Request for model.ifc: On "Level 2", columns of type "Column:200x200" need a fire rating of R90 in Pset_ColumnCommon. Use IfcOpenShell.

First a look at what the model holds.

```python
import ifcopenshell
import ifcopenshell.util.element

model = ifcopenshell.open("model.ifc")
print(model.schema)
storey = next(s for s in model.by_type("IfcBuildingStorey") if s.Name == "Level 2")
columns = [e for e in ifcopenshell.util.element.get_decomposition(storey) if e.is_a("IfcColumn")]
seen = {}
for e in columns:
    element_type = ifcopenshell.util.element.get_type(e)
    key = (element_type.Name if element_type != e and element_type else None, ifcopenshell.util.element.get_pset(e, "Pset_ColumnCommon", "FireRating"))
    seen[key] = seen.get(key, 0) + 1
for (name, value), count in sorted(seen.items(), key=str):
    print(count, "x", name, "|", value)
```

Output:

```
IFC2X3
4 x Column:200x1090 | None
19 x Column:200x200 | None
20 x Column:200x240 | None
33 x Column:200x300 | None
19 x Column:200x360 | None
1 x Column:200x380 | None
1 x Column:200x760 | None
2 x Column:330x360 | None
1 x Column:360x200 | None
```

```python
import ifcopenshell
import ifcopenshell.api.pset
import ifcopenshell.util.element

model = ifcopenshell.open("model.ifc")

storey = next(s for s in model.by_type("IfcBuildingStorey") if s.Name == "Level 2")
columns = [e for e in ifcopenshell.util.element.get_decomposition(storey) if e.is_a("IfcColumn")]

count = 0
for e in columns:
    element_type = ifcopenshell.util.element.get_type(e)
    if element_type in (None, e) or element_type.Name != "Column:200x200":
        continue
    # add_pset returns the element's existing set when there is one.
    pset = ifcopenshell.api.pset.add_pset(model, product=e, name="Pset_ColumnCommon")
    ifcopenshell.api.pset.edit_pset(model, pset=pset, properties={"FireRating": "R90"})
    count += 1

print(count, "columns updated")

model.write("model-out.ifc")
```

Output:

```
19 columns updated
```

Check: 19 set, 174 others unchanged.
